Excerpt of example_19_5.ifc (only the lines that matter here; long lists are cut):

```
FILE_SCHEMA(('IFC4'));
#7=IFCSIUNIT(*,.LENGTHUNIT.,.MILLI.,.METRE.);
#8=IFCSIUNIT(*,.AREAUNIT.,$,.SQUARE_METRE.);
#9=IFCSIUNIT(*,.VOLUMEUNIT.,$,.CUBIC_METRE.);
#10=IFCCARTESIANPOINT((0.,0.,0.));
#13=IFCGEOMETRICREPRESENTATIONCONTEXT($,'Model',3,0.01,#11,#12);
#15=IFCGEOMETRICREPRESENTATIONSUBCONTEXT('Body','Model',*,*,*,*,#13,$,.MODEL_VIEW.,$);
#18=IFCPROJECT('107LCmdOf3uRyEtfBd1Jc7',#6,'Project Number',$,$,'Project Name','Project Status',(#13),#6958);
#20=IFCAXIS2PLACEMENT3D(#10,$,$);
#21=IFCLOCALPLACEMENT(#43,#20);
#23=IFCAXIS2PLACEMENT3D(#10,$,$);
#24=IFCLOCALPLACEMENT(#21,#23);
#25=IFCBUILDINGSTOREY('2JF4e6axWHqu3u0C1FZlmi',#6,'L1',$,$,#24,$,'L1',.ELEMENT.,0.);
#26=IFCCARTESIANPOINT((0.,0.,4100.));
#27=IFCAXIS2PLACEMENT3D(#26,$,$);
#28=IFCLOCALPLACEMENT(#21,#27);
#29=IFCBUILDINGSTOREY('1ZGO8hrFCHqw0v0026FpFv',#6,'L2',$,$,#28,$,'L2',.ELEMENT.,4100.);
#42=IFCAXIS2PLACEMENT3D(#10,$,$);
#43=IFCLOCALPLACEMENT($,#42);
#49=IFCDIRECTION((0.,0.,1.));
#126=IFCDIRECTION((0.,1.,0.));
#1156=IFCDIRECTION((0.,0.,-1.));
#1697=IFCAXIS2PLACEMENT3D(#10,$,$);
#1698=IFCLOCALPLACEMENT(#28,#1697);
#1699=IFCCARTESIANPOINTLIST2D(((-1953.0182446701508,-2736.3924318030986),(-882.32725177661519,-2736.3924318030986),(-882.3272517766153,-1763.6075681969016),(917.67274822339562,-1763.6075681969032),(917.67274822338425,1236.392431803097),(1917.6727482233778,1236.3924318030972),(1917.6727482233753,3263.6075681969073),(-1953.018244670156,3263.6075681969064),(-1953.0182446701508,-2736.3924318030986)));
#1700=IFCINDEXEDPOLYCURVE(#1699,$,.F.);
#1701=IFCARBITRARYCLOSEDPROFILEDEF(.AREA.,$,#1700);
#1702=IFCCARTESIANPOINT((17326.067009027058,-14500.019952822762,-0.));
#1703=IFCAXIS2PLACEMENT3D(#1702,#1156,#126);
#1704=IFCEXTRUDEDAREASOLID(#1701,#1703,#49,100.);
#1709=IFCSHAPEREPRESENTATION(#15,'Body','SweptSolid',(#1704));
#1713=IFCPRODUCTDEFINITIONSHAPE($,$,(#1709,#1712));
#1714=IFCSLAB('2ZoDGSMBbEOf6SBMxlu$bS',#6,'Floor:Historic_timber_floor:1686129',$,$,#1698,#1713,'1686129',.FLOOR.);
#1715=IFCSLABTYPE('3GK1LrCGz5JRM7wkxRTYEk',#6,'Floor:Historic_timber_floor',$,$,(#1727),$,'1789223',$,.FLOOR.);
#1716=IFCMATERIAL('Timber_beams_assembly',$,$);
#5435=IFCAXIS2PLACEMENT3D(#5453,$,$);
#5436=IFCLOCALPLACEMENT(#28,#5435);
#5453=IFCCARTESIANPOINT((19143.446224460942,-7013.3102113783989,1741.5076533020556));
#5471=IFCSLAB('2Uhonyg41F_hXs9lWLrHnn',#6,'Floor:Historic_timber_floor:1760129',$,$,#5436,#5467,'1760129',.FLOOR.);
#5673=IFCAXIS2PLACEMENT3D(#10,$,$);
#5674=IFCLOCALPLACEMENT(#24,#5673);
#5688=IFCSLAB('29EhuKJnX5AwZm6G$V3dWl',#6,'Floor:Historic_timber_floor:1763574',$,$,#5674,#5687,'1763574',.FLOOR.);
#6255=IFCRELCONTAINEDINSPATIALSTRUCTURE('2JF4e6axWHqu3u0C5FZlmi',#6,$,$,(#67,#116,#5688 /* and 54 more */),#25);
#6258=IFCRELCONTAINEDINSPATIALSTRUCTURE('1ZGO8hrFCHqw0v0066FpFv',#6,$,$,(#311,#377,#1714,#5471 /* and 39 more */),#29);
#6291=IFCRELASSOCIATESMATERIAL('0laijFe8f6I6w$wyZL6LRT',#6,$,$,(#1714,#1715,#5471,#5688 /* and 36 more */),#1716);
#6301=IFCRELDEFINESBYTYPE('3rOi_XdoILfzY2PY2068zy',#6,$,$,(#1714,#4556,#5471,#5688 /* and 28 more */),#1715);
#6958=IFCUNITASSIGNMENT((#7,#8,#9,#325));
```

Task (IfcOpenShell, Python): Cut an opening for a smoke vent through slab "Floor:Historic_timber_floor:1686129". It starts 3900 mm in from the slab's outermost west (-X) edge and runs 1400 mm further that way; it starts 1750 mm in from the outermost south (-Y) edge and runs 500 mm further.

```python
import numpy as np
import ifcopenshell
import ifcopenshell.api.feature
import ifcopenshell.api.geometry
import ifcopenshell.api.root
import ifcopenshell.geom
import ifcopenshell.util.placement
import ifcopenshell.util.representation
import ifcopenshell.util.shape
import ifcopenshell.util.unit

model = ifcopenshell.open("example_19_5.ifc")
unit_scale = ifcopenshell.util.unit.calculate_unit_scale(model)
settings = ifcopenshell.geom.settings()


def volume(element):
    """Net volume in cubic metres, openings subtracted."""
    shape = ifcopenshell.geom.create_shape(settings, element)
    return ifcopenshell.util.shape.get_volume(shape.geometry)


slab = model.by_id(1714)
before = volume(slab)

# Extent in the slab's own axes, in metres. The edges named are its -X and -Y sides.
slab_shape = ifcopenshell.geom.create_shape(settings, slab)
vertices = ifcopenshell.util.shape.get_vertices(slab_shape.geometry)
x_min, y_min, bottom = vertices.min(axis=0)
top = vertices[:, 2].max()

opening = ifcopenshell.api.root.create_entity(model, ifc_class="IfcOpeningElement", name="Smoke vent opening", predefined_type="OPENING")
context = ifcopenshell.util.representation.get_context(model, "Model", "Body", "MODEL_VIEW")
width, depth = 1.4, 0.5
outline = [(0.0, 0.0), (width, 0.0), (width, depth), (0.0, depth), (0.0, 0.0)]
# Overshoot both faces by 50 mm so the cut is clean.
shape = ifcopenshell.api.geometry.add_slab_representation(
    model, context=context, depth=top - bottom + 0.1, polyline=outline
)
ifcopenshell.api.geometry.assign_representation(model, product=opening, representation=shape)

matrix = ifcopenshell.util.placement.get_local_placement(slab.ObjectPlacement)
matrix[:, 3] = matrix @ np.append(np.array([x_min + 3.9, y_min + 1.75, bottom - 0.05]) / unit_scale, 1.0)
ifcopenshell.api.geometry.edit_object_placement(model, product=opening, matrix=matrix, is_si=False)
ifcopenshell.api.feature.add_feature(model, feature=opening, element=slab)

after = volume(slab)

print(f"slab volume {before:.3f} -> {after:.3f} m3")

model.write("example_19_5-out.ifc")
```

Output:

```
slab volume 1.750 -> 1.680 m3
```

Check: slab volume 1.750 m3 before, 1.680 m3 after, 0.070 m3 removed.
